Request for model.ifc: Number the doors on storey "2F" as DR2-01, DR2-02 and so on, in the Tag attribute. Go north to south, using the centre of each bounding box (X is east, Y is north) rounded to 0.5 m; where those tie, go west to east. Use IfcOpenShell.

First a look at what the model holds.

```python
import ifcopenshell
import ifcopenshell.util.element
import ifcopenshell.util.placement

model = ifcopenshell.open("model.ifc")
print(model.schema)
storey = next(s for s in model.by_type("IfcBuildingStorey") if s.Name == "2F")
doors = [e for e in ifcopenshell.util.element.get_decomposition(storey) if e.is_a("IfcDoor")]
for e in sorted(doors, key=lambda e: e.id()):
    origin = ifcopenshell.util.placement.get_local_placement(e.ObjectPlacement)[:3, 3]
    print(e.id(), e.Tag, e.Name, origin.round(2) + 0.0, sep=" | ")
```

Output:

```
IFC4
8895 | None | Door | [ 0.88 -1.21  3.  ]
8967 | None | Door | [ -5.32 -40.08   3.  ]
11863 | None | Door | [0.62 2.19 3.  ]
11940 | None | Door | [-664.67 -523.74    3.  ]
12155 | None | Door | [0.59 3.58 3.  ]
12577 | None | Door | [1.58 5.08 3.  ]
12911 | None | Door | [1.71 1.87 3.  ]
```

```python
import ifcopenshell
import ifcopenshell.geom
import ifcopenshell.util.element
import ifcopenshell.util.shape

model = ifcopenshell.open("model.ifc")
settings = ifcopenshell.geom.settings()
settings.set("use-world-coords", True)


def centre(element):
    shape = ifcopenshell.geom.create_shape(settings, element)
    return ifcopenshell.util.shape.get_bbox_centroid(shape.geometry)


storey = next(s for s in model.by_type("IfcBuildingStorey") if s.Name == "2F")
doors = [e for e in ifcopenshell.util.element.get_decomposition(storey) if e.is_a("IfcDoor")]

# Insertion points can sit at a corner or the storey origin, so sort by the geometry (in metres).
centres = {e: centre(e) for e in doors}
doors.sort(key=lambda e: (-round(centres[e][1] / 0.5), centres[e][0]))

for i, e in enumerate(doors, start=1):
    number = f"DR2-{i:02d}"
    e.Tag = number
    print(e.id(), number)

model.write("model-out.ifc")
```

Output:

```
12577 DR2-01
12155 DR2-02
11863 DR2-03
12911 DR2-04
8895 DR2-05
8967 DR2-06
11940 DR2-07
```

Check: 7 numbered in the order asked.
